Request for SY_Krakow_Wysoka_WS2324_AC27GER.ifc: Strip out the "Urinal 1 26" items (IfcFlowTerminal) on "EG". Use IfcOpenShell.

First a look at what the model holds.

```python
import ifcopenshell
import ifcopenshell.util.element

model = ifcopenshell.open("SY_Krakow_Wysoka_WS2324_AC27GER.ifc")
print(model.schema)
storey = next(s for s in model.by_type("IfcBuildingStorey") if s.Name == "EG")
terminals = [e for e in ifcopenshell.util.element.get_decomposition(storey) if e.is_a("IfcFlowTerminal")]
seen = {}
for e in terminals:
    element_type = ifcopenshell.util.element.get_type(e)
    name = element_type.Name if element_type not in (None, e) else None
    seen[name] = seen.get(name, 0) + 1
for name, count in sorted(seen.items(), key=str):
    print(count, "x", name)
```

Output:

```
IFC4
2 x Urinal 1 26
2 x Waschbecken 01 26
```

```python
import ifcopenshell
import ifcopenshell.api.root
import ifcopenshell.util.element

model = ifcopenshell.open("SY_Krakow_Wysoka_WS2324_AC27GER.ifc")

storey = next(s for s in model.by_type("IfcBuildingStorey") if s.Name == "EG")
terminals = [e for e in ifcopenshell.util.element.get_decomposition(storey) if e.is_a("IfcFlowTerminal")]
targets = [e for e in terminals if (t := ifcopenshell.util.element.get_type(e)) not in (None, e) and t.Name == "Urinal 1 26"]

for e in targets:
    ifcopenshell.api.root.remove_product(model, product=e)
print(len(targets), "removed")

model.write("SY_Krakow_Wysoka_WS2324_AC27GER_v2.ifc")
```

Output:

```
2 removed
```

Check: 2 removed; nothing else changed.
